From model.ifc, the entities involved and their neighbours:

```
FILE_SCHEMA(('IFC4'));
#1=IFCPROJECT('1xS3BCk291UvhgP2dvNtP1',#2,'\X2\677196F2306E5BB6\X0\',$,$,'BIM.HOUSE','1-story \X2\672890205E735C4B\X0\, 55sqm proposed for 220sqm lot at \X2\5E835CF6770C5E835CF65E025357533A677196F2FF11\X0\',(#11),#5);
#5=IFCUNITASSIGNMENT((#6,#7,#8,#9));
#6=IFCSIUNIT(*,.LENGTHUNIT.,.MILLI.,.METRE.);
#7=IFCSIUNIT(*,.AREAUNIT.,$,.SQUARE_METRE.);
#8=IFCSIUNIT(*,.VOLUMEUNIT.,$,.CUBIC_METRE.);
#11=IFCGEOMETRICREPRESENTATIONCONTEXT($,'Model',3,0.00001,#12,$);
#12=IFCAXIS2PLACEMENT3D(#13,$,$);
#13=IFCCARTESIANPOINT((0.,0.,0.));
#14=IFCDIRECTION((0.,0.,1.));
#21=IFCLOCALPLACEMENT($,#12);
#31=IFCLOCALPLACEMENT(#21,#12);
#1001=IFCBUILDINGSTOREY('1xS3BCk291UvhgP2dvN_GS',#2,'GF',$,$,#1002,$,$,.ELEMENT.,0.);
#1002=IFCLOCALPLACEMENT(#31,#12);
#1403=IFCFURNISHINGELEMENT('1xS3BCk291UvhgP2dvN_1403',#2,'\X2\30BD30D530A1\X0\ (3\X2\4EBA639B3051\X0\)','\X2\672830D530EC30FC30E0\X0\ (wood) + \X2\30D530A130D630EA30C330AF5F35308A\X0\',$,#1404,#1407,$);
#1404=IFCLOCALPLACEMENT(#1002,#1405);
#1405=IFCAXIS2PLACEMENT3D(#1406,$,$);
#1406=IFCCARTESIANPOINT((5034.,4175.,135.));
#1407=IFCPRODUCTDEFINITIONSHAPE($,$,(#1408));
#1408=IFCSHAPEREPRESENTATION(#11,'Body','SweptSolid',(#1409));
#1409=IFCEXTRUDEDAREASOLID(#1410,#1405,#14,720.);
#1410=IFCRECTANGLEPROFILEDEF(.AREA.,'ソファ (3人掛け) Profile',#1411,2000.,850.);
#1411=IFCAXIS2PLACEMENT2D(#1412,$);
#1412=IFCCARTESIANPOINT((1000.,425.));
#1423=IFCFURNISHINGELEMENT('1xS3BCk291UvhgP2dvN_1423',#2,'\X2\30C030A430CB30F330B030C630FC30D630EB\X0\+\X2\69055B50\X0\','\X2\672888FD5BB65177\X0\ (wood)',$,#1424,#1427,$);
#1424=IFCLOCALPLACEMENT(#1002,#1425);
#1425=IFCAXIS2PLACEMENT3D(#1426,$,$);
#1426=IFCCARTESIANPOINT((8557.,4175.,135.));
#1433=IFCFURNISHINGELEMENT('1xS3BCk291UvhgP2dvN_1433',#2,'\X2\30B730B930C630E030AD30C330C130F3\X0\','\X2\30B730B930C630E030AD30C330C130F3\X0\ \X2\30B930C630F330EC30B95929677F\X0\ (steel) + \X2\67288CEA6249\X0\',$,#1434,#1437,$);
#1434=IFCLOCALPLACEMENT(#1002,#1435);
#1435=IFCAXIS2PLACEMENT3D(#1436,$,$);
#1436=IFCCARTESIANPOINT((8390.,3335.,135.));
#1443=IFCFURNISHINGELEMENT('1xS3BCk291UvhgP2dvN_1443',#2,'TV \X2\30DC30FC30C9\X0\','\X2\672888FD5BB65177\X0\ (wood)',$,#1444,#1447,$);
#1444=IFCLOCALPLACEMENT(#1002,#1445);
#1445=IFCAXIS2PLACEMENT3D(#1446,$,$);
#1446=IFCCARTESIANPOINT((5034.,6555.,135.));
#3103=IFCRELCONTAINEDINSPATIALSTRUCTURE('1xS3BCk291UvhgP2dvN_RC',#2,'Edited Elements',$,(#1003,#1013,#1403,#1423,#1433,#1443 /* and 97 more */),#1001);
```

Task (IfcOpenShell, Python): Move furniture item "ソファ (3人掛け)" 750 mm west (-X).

```python
import ifcopenshell
import ifcopenshell.api.geometry
import ifcopenshell.util.placement

model = ifcopenshell.open("model.ifc")

item = model.by_guid("1xS3BCk291UvhgP2dvN_1403")
matrix = ifcopenshell.util.placement.get_local_placement(item.ObjectPlacement)
matrix[0, 3] -= 750.0
ifcopenshell.api.geometry.edit_object_placement(model, product=item, matrix=matrix, is_si=False)

print(ifcopenshell.util.placement.get_local_placement(item.ObjectPlacement).round(3) + 0.0)

model.write("model-out.ifc")
```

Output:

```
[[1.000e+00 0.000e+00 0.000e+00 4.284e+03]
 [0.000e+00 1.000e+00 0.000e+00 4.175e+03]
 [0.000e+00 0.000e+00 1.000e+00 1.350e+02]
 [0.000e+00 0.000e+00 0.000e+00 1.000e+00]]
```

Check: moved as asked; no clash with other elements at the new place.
